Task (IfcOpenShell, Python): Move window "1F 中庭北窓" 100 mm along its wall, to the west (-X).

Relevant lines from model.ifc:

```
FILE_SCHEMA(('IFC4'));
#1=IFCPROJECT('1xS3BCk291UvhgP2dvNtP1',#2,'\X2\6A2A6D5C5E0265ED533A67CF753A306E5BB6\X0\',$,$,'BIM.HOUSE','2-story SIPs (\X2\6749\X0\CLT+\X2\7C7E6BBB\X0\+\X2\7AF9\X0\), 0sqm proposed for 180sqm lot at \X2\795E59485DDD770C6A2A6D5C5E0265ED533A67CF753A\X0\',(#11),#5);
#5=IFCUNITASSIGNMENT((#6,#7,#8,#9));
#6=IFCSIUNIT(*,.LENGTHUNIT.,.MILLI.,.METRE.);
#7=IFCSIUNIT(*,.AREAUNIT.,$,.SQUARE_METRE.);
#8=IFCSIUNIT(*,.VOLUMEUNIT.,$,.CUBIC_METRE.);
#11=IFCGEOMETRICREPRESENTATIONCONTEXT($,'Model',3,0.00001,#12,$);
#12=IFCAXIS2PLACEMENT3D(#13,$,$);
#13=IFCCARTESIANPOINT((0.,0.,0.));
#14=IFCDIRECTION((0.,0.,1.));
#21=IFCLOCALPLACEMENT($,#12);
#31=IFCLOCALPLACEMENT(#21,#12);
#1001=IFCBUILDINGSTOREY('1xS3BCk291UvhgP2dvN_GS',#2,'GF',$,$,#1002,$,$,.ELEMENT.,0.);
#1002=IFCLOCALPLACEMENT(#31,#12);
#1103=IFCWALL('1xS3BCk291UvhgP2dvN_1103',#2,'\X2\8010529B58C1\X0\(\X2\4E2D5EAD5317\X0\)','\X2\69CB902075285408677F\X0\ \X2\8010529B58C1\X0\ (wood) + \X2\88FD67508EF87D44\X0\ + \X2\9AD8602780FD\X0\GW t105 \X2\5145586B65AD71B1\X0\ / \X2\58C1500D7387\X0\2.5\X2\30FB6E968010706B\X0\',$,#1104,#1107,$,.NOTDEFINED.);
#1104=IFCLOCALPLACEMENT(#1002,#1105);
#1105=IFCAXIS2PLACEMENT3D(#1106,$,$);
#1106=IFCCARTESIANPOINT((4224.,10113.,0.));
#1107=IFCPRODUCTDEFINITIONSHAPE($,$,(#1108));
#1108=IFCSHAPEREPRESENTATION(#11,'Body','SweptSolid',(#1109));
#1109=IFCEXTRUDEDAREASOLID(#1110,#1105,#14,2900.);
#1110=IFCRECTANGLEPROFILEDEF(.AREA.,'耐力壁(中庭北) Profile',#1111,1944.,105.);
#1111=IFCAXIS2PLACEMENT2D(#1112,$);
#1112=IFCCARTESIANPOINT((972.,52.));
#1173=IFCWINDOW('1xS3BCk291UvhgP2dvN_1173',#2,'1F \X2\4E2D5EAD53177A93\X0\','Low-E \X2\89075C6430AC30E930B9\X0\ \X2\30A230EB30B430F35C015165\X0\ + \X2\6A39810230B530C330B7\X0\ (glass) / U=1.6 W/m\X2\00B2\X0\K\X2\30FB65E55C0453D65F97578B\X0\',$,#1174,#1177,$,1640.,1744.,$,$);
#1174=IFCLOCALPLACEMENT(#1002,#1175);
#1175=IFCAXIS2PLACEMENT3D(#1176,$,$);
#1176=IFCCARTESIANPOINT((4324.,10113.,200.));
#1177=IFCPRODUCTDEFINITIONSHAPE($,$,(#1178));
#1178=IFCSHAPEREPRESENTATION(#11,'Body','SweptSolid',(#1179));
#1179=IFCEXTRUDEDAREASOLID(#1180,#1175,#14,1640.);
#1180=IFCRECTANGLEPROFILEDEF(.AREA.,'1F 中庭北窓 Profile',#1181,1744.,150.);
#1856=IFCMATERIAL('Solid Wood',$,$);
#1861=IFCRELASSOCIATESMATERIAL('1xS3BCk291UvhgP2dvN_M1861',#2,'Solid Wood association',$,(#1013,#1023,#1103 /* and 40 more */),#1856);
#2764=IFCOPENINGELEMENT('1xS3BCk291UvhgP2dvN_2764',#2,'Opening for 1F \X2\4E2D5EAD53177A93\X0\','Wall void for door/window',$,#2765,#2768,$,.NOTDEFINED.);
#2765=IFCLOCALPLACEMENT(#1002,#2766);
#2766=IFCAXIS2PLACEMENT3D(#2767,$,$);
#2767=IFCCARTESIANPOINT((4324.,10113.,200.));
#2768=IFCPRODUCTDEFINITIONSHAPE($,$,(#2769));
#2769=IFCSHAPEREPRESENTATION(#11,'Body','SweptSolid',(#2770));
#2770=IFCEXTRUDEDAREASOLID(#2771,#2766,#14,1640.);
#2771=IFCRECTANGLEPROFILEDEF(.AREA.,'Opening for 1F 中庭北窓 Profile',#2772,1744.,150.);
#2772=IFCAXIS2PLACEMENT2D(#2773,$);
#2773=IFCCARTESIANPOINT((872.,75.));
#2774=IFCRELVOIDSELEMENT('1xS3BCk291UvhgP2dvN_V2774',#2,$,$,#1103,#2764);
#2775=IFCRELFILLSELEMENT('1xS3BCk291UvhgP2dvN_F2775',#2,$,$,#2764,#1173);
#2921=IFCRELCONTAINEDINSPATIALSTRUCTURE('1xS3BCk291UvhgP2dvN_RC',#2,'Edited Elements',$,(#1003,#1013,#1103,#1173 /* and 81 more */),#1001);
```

```python
import ifcopenshell
import ifcopenshell.api.geometry
import ifcopenshell.util.placement
import ifcopenshell.util.unit

model = ifcopenshell.open("model.ifc")
unit_scale = ifcopenshell.util.unit.calculate_unit_scale(model)

window = model.by_guid("1xS3BCk291UvhgP2dvN_1173")
opening = window.FillsVoids[0].RelatingOpeningElement
wall = opening.VoidsElements[0].RelatingBuildingElement

wall_matrix = ifcopenshell.util.placement.get_local_placement(wall.ObjectPlacement)
shift = wall_matrix[:3, 0] * -0.1 / unit_scale
before = ifcopenshell.util.placement.get_local_placement(window.ObjectPlacement)[:3, 3].copy()

# The window is not placed relative to its opening, so move both.
for product in (opening, window):
    matrix = ifcopenshell.util.placement.get_local_placement(product.ObjectPlacement)
    matrix[:3, 3] += shift
    ifcopenshell.api.geometry.edit_object_placement(model, product=product, matrix=matrix, is_si=False)

after = ifcopenshell.util.placement.get_local_placement(window.ObjectPlacement)[:3, 3]
print("window moved by", (after - before).round(3) + 0.0)

model.write("model_updated.ifc")
```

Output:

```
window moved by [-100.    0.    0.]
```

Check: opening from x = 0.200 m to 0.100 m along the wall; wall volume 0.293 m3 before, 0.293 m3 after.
